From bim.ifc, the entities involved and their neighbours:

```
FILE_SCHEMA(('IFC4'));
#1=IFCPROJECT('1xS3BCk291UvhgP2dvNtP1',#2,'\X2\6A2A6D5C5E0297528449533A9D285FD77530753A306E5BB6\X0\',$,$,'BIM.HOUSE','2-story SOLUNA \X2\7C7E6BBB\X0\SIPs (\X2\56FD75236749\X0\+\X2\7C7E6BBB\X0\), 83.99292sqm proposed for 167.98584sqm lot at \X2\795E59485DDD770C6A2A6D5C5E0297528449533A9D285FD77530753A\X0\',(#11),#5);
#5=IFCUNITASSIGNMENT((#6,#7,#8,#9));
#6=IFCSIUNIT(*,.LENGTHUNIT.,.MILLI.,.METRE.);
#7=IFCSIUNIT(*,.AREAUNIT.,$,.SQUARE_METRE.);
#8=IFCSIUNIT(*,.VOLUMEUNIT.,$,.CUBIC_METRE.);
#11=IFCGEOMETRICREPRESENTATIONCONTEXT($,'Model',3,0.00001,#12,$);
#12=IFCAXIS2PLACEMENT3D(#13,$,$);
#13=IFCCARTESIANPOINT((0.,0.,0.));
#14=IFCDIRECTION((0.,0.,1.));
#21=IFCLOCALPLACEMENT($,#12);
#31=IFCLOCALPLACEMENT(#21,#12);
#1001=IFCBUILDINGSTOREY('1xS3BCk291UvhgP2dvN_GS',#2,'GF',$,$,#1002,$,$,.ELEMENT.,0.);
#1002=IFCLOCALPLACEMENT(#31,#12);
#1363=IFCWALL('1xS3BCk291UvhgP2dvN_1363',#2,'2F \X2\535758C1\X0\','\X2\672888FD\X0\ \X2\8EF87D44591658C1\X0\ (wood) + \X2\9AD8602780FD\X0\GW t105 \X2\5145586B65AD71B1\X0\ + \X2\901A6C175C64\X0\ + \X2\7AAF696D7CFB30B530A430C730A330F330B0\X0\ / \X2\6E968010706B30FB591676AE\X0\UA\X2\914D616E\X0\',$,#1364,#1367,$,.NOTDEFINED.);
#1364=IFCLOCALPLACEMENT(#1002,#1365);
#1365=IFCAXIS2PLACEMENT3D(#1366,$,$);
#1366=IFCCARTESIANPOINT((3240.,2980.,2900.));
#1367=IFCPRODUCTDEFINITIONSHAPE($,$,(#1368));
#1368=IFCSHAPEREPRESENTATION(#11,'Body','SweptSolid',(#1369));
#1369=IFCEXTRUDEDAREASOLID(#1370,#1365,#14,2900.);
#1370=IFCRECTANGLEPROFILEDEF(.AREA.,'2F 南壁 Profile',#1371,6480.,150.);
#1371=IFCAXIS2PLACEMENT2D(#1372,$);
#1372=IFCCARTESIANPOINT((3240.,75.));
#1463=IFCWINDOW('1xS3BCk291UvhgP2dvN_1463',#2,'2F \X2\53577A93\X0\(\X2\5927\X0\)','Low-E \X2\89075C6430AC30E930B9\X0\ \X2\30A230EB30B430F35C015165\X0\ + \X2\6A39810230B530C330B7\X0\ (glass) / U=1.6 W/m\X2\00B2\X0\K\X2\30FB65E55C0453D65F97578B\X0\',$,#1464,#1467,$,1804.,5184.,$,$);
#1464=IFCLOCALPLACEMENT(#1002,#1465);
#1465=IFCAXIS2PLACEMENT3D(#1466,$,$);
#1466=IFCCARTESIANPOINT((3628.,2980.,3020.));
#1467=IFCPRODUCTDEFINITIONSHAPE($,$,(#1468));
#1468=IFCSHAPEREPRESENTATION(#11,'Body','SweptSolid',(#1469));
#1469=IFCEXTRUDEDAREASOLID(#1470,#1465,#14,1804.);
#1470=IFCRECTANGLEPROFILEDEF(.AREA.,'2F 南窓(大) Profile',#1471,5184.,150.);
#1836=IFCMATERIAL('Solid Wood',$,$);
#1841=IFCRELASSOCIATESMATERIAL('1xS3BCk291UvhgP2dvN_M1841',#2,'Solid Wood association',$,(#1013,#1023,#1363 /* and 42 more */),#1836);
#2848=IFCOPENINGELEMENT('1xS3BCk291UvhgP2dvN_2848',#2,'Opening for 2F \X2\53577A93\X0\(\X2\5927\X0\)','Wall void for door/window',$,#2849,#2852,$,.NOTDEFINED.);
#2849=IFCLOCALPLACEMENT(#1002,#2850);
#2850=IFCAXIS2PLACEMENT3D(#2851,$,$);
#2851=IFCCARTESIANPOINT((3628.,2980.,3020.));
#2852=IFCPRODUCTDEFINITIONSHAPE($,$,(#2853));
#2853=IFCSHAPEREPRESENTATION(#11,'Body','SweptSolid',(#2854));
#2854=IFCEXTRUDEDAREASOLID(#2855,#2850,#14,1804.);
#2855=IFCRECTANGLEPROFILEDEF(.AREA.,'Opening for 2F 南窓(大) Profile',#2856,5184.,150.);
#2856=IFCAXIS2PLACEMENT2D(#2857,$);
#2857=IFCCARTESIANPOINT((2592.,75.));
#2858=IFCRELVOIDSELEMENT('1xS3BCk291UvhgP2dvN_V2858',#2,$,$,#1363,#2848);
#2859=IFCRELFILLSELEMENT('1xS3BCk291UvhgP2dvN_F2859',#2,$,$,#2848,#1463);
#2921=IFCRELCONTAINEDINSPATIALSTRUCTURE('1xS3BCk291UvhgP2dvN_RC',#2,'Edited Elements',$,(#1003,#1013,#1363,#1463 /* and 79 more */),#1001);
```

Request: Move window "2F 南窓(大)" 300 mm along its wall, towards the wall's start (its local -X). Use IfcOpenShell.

```python
import ifcopenshell
import ifcopenshell.api.geometry
import ifcopenshell.util.placement

model = ifcopenshell.open("bim.ifc")

window = model.by_id(1463)
opening = window.FillsVoids[0].RelatingOpeningElement
wall = opening.VoidsElements[0].RelatingBuildingElement

wall_matrix = ifcopenshell.util.placement.get_local_placement(wall.ObjectPlacement)
shift = wall_matrix[:3, 0] * -300.0
before = ifcopenshell.util.placement.get_local_placement(window.ObjectPlacement)[:3, 3].copy()

# The window is not placed relative to its opening, so move both.
for product in (opening, window):
    matrix = ifcopenshell.util.placement.get_local_placement(product.ObjectPlacement)
    matrix[:3, 3] += shift
    ifcopenshell.api.geometry.edit_object_placement(model, product=product, matrix=matrix, is_si=False)

after = ifcopenshell.util.placement.get_local_placement(window.ObjectPlacement)[:3, 3]
print("window moved by", (after - before).round(3) + 0.0)

model.write("bim-out.ifc")
```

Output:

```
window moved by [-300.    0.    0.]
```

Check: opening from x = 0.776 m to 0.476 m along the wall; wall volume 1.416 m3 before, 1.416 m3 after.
